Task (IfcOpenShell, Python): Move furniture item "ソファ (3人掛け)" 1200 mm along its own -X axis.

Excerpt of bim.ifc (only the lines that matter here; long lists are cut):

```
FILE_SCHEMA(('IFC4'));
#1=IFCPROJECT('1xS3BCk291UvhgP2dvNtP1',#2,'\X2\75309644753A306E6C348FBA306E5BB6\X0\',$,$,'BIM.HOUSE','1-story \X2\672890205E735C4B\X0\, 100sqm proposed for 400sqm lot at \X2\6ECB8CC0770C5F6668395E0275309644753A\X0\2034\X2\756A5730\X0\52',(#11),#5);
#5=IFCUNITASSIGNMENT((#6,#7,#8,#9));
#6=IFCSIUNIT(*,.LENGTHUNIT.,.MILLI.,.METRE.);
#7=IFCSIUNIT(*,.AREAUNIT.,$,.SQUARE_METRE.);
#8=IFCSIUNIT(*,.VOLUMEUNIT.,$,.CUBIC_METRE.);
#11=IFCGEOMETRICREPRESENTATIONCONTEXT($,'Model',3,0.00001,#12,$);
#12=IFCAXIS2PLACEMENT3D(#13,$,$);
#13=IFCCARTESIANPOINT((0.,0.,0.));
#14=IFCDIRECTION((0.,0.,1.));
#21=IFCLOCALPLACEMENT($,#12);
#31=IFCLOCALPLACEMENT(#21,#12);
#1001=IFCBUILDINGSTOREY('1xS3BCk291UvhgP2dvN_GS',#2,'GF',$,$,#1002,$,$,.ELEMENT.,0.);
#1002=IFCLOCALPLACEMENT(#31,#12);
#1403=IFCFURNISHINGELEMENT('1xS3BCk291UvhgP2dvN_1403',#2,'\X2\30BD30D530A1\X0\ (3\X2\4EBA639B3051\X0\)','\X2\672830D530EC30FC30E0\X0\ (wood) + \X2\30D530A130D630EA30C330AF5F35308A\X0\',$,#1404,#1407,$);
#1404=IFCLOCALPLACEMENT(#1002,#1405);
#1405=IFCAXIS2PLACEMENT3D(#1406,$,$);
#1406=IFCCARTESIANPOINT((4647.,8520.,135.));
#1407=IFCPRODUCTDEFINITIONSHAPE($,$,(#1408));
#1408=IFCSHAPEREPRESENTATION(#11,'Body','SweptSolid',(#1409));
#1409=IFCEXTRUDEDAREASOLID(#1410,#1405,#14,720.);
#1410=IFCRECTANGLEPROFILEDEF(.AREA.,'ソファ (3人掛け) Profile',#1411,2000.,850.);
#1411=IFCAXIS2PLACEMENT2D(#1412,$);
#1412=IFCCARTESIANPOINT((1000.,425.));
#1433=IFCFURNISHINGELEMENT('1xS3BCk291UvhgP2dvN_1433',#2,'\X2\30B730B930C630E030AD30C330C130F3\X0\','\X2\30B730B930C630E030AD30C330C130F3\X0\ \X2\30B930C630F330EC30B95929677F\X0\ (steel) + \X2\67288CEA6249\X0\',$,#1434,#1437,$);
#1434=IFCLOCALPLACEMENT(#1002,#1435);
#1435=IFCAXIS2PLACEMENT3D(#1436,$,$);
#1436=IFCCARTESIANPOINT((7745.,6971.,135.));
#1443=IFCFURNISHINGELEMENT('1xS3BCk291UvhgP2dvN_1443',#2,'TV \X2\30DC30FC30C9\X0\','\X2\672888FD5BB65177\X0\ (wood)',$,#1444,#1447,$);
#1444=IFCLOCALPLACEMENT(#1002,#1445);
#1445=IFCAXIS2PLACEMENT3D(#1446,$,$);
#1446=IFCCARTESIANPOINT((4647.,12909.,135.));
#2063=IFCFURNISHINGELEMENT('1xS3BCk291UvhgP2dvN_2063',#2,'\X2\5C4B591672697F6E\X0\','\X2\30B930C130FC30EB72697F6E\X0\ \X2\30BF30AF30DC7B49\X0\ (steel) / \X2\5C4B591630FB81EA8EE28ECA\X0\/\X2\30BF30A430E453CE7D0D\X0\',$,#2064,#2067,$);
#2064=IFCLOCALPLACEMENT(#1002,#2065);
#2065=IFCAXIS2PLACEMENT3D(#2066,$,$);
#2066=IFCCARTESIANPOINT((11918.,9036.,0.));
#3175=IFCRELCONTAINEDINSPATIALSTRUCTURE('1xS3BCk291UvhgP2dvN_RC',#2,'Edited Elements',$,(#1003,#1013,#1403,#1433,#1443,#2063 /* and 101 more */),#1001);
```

```python
import ifcopenshell
import ifcopenshell.api.geometry
import ifcopenshell.util.placement

model = ifcopenshell.open("bim.ifc")

item = model.by_guid("1xS3BCk291UvhgP2dvN_1403")
matrix = ifcopenshell.util.placement.get_local_placement(item.ObjectPlacement)
matrix[:3, 3] -= matrix[:3, 0] * 1200.0
ifcopenshell.api.geometry.edit_object_placement(model, product=item, matrix=matrix, is_si=False)

print(ifcopenshell.util.placement.get_local_placement(item.ObjectPlacement).round(3) + 0.0)

model.write("bim_updated.ifc")
```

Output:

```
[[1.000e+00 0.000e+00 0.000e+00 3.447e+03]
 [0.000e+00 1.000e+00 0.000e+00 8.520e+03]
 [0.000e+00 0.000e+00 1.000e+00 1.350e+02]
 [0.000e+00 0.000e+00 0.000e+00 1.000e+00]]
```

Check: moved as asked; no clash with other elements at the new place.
